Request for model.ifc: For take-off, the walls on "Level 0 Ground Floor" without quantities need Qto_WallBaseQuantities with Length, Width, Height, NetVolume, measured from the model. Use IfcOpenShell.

First a look at what the model holds.

```python
import ifcopenshell
import ifcopenshell.util.element
import ifcopenshell.util.unit

model = ifcopenshell.open("model.ifc")
print(model.schema)
for unit_type in ("LENGTHUNIT", "AREAUNIT", "VOLUMEUNIT"):
    print(unit_type, ifcopenshell.util.unit.calculate_unit_scale(model, unit_type))
storey = next(s for s in model.by_type("IfcBuildingStorey") if s.Name == "Level 0 Ground Floor")
walls = [e for e in ifcopenshell.util.element.get_decomposition(storey) if e.is_a("IfcWall")]
for e in sorted(walls, key=lambda e: e.id()):
    print(e.id(), e.is_a(), e.Name, list(ifcopenshell.util.element.get_psets(e, qtos_only=True)), sep=" | ")
```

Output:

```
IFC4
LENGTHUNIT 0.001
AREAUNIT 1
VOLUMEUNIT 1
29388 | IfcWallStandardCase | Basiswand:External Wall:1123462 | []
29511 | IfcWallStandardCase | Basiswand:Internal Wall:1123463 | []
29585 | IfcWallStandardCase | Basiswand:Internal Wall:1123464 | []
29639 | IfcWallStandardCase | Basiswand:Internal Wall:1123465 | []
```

```python
import ifcopenshell
import ifcopenshell.api.pset
import ifcopenshell.geom
import ifcopenshell.util.element
import ifcopenshell.util.shape
import ifcopenshell.util.unit

model = ifcopenshell.open("model.ifc")
unit_scale = ifcopenshell.util.unit.calculate_unit_scale(model)
volume_scale = ifcopenshell.util.unit.calculate_unit_scale(model, "VOLUMEUNIT")
settings = ifcopenshell.geom.settings()

storey = next(s for s in model.by_type("IfcBuildingStorey") if s.Name == "Level 0 Ground Floor")
walls = [e for e in ifcopenshell.util.element.get_decomposition(storey) if e.is_a("IfcWall")]

for e in sorted(walls, key=lambda e: e.id()):
    if ifcopenshell.util.element.get_psets(e, qtos_only=True, should_inherit=False):
        continue
    # Geometry comes back in metres, in the element's own axes.
    shape = ifcopenshell.geom.create_shape(settings, e)
    values = {
        "Length": ifcopenshell.util.shape.get_x(shape.geometry) / unit_scale,
        "Width": ifcopenshell.util.shape.get_y(shape.geometry) / unit_scale,
        "Height": ifcopenshell.util.shape.get_z(shape.geometry) / unit_scale,
        "NetVolume": ifcopenshell.util.shape.get_volume(shape.geometry) / volume_scale,
    }
    qto = ifcopenshell.api.pset.add_qto(model, product=e, name="Qto_WallBaseQuantities")
    ifcopenshell.api.pset.edit_qto(model, qto=qto, properties=values)
    print(e.id(), {k: round(v, 3) for k, v in values.items()})

model.write("model_v2.ifc")
```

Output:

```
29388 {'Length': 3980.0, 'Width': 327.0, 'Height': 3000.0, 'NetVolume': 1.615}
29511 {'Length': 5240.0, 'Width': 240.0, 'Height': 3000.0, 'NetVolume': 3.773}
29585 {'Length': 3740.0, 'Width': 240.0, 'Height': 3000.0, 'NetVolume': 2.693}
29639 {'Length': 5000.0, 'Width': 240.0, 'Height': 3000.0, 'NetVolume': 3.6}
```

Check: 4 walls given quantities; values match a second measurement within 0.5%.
